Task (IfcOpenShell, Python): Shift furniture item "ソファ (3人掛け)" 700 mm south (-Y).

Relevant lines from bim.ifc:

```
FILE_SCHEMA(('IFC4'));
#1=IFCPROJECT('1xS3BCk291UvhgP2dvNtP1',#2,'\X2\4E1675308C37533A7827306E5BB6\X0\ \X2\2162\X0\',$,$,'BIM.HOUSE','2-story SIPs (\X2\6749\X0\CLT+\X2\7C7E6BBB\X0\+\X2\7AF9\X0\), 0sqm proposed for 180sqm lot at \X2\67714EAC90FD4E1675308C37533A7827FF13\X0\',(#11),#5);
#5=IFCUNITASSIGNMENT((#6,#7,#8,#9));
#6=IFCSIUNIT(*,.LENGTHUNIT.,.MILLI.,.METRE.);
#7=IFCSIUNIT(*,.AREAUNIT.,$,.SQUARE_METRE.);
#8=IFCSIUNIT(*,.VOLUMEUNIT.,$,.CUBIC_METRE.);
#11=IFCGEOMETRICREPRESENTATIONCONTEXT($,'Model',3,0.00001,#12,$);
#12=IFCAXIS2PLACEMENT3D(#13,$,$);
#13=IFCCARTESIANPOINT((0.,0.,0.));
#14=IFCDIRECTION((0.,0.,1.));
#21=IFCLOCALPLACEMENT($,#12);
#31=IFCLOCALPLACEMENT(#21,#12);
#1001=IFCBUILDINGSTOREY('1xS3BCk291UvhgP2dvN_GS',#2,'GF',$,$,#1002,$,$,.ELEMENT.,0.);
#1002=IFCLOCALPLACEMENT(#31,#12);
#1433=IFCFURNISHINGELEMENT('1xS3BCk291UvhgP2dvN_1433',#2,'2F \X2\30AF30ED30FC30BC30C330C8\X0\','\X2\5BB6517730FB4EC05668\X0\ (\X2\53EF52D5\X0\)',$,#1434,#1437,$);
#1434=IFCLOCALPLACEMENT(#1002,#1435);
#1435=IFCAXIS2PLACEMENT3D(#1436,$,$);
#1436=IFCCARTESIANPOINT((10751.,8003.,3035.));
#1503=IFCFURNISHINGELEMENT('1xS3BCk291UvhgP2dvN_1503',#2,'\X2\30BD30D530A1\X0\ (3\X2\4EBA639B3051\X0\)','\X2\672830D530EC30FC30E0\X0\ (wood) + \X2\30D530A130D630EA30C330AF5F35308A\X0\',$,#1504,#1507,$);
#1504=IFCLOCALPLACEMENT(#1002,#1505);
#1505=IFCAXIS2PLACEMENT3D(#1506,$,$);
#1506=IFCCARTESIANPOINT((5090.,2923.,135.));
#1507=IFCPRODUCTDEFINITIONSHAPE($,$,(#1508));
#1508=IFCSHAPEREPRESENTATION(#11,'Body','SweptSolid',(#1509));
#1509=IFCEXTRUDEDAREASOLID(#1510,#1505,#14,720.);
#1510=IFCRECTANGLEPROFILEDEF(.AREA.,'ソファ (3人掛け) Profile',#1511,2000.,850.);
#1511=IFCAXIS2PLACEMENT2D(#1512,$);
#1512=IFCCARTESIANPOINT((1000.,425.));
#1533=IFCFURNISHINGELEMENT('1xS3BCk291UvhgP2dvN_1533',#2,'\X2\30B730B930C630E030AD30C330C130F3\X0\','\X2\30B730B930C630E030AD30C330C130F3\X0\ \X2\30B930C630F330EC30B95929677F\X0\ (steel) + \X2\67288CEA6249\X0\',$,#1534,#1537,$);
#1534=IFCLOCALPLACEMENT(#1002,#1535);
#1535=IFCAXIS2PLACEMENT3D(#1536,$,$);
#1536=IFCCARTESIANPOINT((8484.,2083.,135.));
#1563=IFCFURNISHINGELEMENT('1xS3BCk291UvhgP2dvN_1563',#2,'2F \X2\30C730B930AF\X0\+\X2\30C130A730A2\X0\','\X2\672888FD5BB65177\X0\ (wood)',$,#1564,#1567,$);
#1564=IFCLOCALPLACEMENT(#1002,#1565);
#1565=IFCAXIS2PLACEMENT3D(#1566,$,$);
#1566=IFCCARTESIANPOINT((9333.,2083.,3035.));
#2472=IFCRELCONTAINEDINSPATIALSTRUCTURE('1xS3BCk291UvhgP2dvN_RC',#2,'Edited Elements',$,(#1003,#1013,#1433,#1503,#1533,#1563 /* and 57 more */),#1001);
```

```python
import ifcopenshell
import ifcopenshell.api.geometry
import ifcopenshell.util.placement

model = ifcopenshell.open("bim.ifc")

item = model.by_guid("1xS3BCk291UvhgP2dvN_1503")
matrix = ifcopenshell.util.placement.get_local_placement(item.ObjectPlacement)
matrix[1, 3] -= 700.0
ifcopenshell.api.geometry.edit_object_placement(model, product=item, matrix=matrix, is_si=False)

print(ifcopenshell.util.placement.get_local_placement(item.ObjectPlacement).round(3) + 0.0)

model.write("bim_edited.ifc")
```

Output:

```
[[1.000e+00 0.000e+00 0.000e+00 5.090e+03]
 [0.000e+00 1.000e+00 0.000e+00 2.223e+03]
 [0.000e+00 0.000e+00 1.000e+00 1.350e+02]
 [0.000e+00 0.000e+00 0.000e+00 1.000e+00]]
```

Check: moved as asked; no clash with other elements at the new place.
